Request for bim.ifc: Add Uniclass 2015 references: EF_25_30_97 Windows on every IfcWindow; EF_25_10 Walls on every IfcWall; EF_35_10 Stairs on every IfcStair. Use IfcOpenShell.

First a look at what the model holds.

```python
import ifcopenshell

model = ifcopenshell.open("bim.ifc")
print(model.schema)
print("classifications:", [c.Name for c in model.by_type("IfcClassification")])
for ifc_class in ("IfcDoor", "IfcRoof", "IfcStair", "IfcWall", "IfcWindow"):
    print(ifc_class, len(model.by_type(ifc_class)))
```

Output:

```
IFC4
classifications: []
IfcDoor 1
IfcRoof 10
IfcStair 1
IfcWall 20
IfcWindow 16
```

```python
import ifcopenshell
import ifcopenshell.api.classification

model = ifcopenshell.open("bim.ifc")

system = ifcopenshell.api.classification.add_classification(model, classification="Uniclass 2015")

codes = {
    "IfcWindow": ("EF_25_30_97", "Windows"),
    "IfcWall": ("EF_25_10", "Walls"),
    "IfcStair": ("EF_35_10", "Stairs"),
}
for ifc_class, (code, name) in codes.items():
    products = model.by_type(ifc_class)
    ifcopenshell.api.classification.add_reference(
        model, products=products, classification=system, identification=code, name=name
    )
    print(code, len(products))

model.write("bim_rev.ifc")
```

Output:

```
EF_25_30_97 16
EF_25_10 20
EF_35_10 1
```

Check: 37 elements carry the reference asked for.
